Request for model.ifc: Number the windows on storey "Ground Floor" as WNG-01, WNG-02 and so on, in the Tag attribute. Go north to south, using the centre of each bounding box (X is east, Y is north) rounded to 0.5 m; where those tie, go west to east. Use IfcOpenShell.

First a look at what the model holds.

```python
import ifcopenshell
import ifcopenshell.util.element
import ifcopenshell.util.placement

model = ifcopenshell.open("model.ifc")
print(model.schema)
storey = next(s for s in model.by_type("IfcBuildingStorey") if s.Name == "Ground Floor")
windows = [e for e in ifcopenshell.util.element.get_decomposition(storey) if e.is_a("IfcWindow")]
for e in sorted(windows, key=lambda e: e.id()):
    origin = ifcopenshell.util.placement.get_local_placement(e.ObjectPlacement)[:3, 3]
    print(e.id(), e.Tag, e.Name, origin.round(2) + 0.0, sep=" | ")
```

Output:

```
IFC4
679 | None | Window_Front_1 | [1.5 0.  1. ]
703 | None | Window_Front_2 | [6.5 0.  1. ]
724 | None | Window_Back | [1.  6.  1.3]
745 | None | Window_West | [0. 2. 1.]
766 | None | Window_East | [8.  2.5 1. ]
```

```python
import ifcopenshell
import ifcopenshell.geom
import ifcopenshell.util.element
import ifcopenshell.util.shape

model = ifcopenshell.open("model.ifc")
settings = ifcopenshell.geom.settings()
settings.set("use-world-coords", True)


def centre(element):
    shape = ifcopenshell.geom.create_shape(settings, element)
    return ifcopenshell.util.shape.get_bbox_centroid(shape.geometry)


storey = next(s for s in model.by_type("IfcBuildingStorey") if s.Name == "Ground Floor")
windows = [e for e in ifcopenshell.util.element.get_decomposition(storey) if e.is_a("IfcWindow")]

# Insertion points can sit at a corner or the storey origin, so sort by the geometry (in metres).
centres = {e: centre(e) for e in windows}
windows.sort(key=lambda e: (-round(centres[e][1] / 0.5), centres[e][0]))

for i, e in enumerate(windows, start=1):
    number = f"WNG-{i:02d}"
    e.Tag = number
    print(e.id(), number)

model.write("model_edited.ifc")
```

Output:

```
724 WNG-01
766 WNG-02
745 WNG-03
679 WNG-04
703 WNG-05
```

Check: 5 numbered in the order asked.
